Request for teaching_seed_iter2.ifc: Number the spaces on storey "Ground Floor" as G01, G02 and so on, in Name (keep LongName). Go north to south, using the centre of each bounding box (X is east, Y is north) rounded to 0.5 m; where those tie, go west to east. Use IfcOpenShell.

First a look at what the model holds.

```python
import ifcopenshell
import ifcopenshell.util.element
import ifcopenshell.util.placement

model = ifcopenshell.open("teaching_seed_iter2.ifc")
print(model.schema)
storey = next(s for s in model.by_type("IfcBuildingStorey") if s.Name == "Ground Floor")
spaces = [e for e in ifcopenshell.util.element.get_decomposition(storey) if e.is_a("IfcSpace")]
for e in sorted(spaces, key=lambda e: e.id()):
    origin = ifcopenshell.util.placement.get_local_placement(e.ObjectPlacement)[:3, 3]
    print(e.id(), e.Name, e.LongName, origin.round(2) + 0.0, sep=" | ")
```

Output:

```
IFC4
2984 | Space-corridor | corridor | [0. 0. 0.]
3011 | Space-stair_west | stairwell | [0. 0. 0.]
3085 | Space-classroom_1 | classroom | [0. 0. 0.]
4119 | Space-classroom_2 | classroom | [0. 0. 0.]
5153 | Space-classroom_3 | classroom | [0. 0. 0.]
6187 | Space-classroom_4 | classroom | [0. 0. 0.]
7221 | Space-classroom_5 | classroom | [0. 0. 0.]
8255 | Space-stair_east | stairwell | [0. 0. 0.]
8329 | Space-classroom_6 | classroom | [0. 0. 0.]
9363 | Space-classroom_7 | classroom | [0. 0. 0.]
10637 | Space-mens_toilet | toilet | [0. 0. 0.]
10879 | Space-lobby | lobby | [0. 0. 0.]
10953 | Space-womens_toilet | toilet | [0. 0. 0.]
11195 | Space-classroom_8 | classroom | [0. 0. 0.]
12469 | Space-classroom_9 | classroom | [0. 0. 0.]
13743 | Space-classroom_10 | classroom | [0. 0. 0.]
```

```python
import ifcopenshell
import ifcopenshell.geom
import ifcopenshell.util.element
import ifcopenshell.util.shape

model = ifcopenshell.open("teaching_seed_iter2.ifc")
settings = ifcopenshell.geom.settings()
settings.set("use-world-coords", True)


def centre(element):
    shape = ifcopenshell.geom.create_shape(settings, element)
    return ifcopenshell.util.shape.get_bbox_centroid(shape.geometry)


storey = next(s for s in model.by_type("IfcBuildingStorey") if s.Name == "Ground Floor")
spaces = [e for e in ifcopenshell.util.element.get_decomposition(storey) if e.is_a("IfcSpace")]

# Insertion points can sit at a corner or the storey origin, so sort by the geometry (in metres).
centres = {e: centre(e) for e in spaces}
spaces.sort(key=lambda e: (-round(centres[e][1] / 0.5), centres[e][0]))

for i, e in enumerate(spaces, start=1):
    number = f"G{i:02d}"
    e.Name = number
    print(e.id(), number)

model.write("teaching_seed_iter2_edited.ifc")
```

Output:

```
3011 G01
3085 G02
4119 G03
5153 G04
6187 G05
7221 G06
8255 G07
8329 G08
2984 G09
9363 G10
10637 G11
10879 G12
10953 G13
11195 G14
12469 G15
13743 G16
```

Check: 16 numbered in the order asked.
